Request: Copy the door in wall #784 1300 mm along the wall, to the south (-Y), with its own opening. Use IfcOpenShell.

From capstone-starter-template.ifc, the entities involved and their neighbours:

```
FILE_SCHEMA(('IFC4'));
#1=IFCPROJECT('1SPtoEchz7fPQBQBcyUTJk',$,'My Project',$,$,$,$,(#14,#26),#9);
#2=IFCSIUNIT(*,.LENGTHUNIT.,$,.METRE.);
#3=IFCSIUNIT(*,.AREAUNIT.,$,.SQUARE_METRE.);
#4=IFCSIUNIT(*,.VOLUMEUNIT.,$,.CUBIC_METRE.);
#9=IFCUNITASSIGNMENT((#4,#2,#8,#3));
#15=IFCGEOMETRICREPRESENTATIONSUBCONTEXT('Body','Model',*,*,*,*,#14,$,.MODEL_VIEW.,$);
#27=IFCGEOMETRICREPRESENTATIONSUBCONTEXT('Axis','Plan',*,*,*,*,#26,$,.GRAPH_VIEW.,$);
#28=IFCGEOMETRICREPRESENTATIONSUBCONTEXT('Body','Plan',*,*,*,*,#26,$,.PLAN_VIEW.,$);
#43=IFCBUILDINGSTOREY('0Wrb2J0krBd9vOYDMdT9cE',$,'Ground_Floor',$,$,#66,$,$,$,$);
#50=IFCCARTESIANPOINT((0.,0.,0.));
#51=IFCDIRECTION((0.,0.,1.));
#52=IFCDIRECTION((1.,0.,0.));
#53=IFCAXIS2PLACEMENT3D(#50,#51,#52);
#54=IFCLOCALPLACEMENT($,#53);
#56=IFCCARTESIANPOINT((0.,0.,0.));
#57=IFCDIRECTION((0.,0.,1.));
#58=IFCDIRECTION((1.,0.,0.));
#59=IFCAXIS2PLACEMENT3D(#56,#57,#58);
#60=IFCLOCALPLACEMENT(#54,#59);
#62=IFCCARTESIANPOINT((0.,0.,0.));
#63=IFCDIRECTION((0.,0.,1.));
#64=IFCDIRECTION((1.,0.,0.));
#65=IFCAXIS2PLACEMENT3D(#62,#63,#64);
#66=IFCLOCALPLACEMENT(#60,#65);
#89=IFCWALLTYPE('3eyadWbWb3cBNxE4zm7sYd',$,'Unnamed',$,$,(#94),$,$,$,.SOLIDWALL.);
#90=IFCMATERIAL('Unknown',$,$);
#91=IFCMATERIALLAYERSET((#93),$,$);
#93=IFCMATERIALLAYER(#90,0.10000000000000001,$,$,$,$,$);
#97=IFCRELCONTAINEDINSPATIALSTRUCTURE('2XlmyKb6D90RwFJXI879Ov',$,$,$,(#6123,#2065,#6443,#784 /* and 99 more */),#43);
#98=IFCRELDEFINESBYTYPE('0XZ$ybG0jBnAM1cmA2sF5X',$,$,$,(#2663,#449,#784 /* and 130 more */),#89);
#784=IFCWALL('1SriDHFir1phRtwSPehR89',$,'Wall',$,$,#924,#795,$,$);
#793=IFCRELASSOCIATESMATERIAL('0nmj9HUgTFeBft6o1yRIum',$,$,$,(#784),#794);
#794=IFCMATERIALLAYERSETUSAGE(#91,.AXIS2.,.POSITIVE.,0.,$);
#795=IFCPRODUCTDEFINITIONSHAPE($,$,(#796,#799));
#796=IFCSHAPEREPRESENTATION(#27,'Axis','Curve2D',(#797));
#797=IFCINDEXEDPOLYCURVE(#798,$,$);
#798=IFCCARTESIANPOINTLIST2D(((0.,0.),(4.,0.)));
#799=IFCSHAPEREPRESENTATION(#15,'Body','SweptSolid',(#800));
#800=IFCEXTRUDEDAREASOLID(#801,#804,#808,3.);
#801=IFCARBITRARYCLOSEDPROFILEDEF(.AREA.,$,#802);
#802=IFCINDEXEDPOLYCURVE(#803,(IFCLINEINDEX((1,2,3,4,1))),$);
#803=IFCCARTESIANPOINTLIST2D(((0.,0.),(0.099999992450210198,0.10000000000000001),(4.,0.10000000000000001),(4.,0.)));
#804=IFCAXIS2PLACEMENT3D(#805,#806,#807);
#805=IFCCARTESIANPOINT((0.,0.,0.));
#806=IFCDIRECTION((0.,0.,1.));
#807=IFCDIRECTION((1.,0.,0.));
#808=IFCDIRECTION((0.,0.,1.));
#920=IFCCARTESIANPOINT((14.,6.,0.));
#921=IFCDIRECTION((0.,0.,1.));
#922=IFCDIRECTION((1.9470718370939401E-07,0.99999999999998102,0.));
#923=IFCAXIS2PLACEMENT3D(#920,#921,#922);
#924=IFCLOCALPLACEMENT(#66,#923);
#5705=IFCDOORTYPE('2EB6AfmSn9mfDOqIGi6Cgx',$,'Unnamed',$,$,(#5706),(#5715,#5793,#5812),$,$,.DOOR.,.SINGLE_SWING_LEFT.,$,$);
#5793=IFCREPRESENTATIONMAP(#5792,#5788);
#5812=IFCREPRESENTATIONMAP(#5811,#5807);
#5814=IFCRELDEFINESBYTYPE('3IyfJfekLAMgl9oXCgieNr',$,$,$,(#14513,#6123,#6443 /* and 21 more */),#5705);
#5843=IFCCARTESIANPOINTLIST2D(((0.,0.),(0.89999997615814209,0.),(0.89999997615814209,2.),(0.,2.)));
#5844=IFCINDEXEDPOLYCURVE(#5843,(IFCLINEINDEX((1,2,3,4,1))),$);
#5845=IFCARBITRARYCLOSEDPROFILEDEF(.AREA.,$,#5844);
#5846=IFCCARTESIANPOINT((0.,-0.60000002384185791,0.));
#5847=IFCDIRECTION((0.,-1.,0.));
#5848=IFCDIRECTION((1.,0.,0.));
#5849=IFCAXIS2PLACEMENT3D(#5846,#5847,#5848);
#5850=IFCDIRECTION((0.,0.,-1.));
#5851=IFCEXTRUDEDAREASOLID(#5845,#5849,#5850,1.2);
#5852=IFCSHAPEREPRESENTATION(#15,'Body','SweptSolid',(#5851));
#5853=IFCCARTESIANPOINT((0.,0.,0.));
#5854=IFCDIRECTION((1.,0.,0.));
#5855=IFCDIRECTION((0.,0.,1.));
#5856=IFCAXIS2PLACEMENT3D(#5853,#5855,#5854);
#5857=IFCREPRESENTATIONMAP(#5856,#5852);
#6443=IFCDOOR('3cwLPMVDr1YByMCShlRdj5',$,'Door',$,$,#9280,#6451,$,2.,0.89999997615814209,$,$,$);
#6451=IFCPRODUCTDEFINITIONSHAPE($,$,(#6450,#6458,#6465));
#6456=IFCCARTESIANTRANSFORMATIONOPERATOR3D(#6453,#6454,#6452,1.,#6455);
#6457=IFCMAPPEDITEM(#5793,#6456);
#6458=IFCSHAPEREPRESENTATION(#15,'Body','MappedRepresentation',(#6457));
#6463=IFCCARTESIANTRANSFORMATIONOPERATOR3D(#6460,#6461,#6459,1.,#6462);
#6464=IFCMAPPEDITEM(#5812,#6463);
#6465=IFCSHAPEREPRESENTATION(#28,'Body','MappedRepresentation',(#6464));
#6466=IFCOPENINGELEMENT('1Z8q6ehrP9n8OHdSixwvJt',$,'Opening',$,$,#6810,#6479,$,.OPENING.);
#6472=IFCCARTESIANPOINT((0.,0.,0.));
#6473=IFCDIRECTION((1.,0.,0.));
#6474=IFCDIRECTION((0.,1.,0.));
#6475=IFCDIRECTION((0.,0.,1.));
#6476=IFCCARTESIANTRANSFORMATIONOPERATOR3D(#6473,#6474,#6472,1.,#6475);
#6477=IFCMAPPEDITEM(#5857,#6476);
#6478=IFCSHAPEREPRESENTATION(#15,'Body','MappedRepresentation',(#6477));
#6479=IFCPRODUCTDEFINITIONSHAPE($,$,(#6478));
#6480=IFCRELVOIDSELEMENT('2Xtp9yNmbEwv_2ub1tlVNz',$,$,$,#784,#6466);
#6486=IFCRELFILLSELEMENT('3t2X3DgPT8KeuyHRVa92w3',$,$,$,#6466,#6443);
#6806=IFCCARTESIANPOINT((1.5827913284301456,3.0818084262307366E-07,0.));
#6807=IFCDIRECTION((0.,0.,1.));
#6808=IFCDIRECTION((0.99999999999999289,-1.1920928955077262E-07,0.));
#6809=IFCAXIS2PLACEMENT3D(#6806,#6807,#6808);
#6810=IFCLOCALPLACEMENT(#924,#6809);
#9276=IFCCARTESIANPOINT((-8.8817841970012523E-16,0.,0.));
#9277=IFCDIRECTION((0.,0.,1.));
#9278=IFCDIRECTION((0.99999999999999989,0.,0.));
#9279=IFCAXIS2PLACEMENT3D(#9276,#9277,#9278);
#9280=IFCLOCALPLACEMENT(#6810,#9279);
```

```python
import ifcopenshell
import ifcopenshell.api.feature
import ifcopenshell.api.geometry
import ifcopenshell.api.root
import ifcopenshell.geom
import ifcopenshell.util.element
import ifcopenshell.util.placement
import ifcopenshell.util.shape
import ifcopenshell.util.unit

model = ifcopenshell.open("capstone-starter-template.ifc")
unit_scale = ifcopenshell.util.unit.calculate_unit_scale(model)
settings = ifcopenshell.geom.settings()


def volume(element):
    """Net volume in cubic metres, openings subtracted."""
    shape = ifcopenshell.geom.create_shape(settings, element)
    return ifcopenshell.util.shape.get_volume(shape.geometry)


door = model.by_guid("3cwLPMVDr1YByMCShlRdj5")
opening = door.FillsVoids[0].RelatingOpeningElement
wall = opening.VoidsElements[0].RelatingBuildingElement
before = volume(wall)
shift = ifcopenshell.util.placement.get_local_placement(wall.ObjectPlacement)[:3, 0] * -1.3 / unit_scale

# copy_class copies the void relationship, type, container and properties, but no geometry.
new_opening = ifcopenshell.api.root.copy_class(model, product=opening)
new_opening.Representation = ifcopenshell.util.element.copy_deep(
    model, opening.Representation, exclude=["IfcGeometricRepresentationContext", "IfcRepresentationMap"]
)
new_door = ifcopenshell.api.root.copy_class(model, product=door)
new_door.Representation = ifcopenshell.util.element.copy_deep(
    model, door.Representation, exclude=["IfcGeometricRepresentationContext", "IfcRepresentationMap"]
)
ifcopenshell.api.feature.add_filling(model, opening=new_opening, element=new_door)

for old, new in ((opening, new_opening), (door, new_door)):
    matrix = ifcopenshell.util.placement.get_local_placement(old.ObjectPlacement)
    matrix[:3, 3] += shift
    ifcopenshell.api.geometry.edit_object_placement(model, product=new, matrix=matrix, is_si=False)

after = volume(wall)

print(f"wall volume {before:.3f} -> {after:.3f} m3")

model.write("capstone-starter-template_rev.ifc")
```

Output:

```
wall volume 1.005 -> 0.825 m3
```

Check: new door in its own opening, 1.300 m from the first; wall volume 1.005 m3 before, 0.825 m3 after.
